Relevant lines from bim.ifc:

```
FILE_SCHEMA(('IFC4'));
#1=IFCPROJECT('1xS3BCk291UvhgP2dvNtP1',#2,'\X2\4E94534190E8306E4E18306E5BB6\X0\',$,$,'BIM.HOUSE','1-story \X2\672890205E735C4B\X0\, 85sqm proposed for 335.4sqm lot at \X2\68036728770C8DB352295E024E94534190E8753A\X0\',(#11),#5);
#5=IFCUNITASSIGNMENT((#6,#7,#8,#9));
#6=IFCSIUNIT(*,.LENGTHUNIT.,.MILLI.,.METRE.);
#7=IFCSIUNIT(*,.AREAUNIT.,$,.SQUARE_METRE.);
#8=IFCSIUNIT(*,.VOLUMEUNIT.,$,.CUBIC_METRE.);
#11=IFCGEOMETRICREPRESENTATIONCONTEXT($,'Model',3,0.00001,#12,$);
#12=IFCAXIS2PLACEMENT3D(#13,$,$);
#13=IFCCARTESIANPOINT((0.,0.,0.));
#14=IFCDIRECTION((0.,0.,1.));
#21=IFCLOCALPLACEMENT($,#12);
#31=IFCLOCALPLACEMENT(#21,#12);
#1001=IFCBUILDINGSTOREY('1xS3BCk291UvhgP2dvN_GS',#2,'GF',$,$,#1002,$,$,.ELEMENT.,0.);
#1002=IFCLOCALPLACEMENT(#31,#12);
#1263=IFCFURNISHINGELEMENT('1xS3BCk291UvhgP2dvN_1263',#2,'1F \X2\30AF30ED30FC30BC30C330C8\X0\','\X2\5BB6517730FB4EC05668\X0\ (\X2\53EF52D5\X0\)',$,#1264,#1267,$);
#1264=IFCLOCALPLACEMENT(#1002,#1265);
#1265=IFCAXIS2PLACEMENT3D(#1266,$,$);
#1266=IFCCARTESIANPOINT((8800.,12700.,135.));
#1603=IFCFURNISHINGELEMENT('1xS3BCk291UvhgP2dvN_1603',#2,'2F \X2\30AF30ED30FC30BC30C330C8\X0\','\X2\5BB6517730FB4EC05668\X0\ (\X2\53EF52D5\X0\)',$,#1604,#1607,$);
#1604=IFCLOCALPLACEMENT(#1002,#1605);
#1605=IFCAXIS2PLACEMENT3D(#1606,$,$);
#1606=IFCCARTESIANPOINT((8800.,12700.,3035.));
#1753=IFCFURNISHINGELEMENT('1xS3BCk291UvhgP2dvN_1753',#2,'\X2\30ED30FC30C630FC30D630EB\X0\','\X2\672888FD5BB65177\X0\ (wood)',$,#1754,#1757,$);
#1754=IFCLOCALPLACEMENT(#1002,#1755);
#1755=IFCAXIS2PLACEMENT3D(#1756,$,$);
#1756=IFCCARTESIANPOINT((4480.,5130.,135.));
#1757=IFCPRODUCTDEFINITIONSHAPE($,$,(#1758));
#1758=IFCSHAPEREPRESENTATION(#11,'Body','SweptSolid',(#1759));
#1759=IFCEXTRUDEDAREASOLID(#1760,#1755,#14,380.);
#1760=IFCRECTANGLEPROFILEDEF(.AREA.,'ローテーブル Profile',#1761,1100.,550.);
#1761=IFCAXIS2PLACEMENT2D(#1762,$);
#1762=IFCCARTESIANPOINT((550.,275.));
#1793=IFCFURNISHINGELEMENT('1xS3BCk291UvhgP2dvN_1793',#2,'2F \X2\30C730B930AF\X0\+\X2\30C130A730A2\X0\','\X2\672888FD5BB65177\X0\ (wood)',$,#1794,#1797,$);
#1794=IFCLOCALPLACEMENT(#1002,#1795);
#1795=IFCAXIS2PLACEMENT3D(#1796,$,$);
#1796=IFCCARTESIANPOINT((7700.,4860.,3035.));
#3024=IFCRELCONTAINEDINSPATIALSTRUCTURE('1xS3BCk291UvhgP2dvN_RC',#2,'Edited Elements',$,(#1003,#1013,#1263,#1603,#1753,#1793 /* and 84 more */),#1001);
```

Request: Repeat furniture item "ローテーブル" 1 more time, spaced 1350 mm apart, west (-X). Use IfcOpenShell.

```python
import numpy as np
import ifcopenshell
import ifcopenshell.api.geometry
import ifcopenshell.api.root
import ifcopenshell.util.element
import ifcopenshell.util.placement
import ifcopenshell.util.unit

model = ifcopenshell.open("bim.ifc")
unit_scale = ifcopenshell.util.unit.calculate_unit_scale(model)


def reuse_history(source, copy):
    """copy_class also copies each property set's owner history, people and application; keep the originals."""
    for rel in copy.IsDefinedBy:
        if rel.is_a("IfcRelDefinesByProperties") and (history := rel.RelatingPropertyDefinition.OwnerHistory):
            rel.RelatingPropertyDefinition.OwnerHistory = source.OwnerHistory
            ifcopenshell.util.element.remove_deep2(model, history)


source = model.by_guid("1xS3BCk291UvhgP2dvN_1753")
base = ifcopenshell.util.placement.get_local_placement(source.ObjectPlacement)
step = np.array([-1.0, 0.0, 0.0]) * 1.35 / unit_scale

for i in range(1, 2):
    copy = ifcopenshell.api.root.copy_class(model, product=source)
    copy.Representation = ifcopenshell.util.element.copy_deep(
        model, source.Representation, exclude=["IfcGeometricRepresentationContext", "IfcRepresentationMap"]
    )
    reuse_history(source, copy)
    matrix = base.copy()
    matrix[:3, 3] += i * step
    print("added at", matrix[:3, 3].round(3) + 0.0)
    ifcopenshell.api.geometry.edit_object_placement(model, product=copy, matrix=matrix, is_si=False)

model.write("bim_edited.ifc")
```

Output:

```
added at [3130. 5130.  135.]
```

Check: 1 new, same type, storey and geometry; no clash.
